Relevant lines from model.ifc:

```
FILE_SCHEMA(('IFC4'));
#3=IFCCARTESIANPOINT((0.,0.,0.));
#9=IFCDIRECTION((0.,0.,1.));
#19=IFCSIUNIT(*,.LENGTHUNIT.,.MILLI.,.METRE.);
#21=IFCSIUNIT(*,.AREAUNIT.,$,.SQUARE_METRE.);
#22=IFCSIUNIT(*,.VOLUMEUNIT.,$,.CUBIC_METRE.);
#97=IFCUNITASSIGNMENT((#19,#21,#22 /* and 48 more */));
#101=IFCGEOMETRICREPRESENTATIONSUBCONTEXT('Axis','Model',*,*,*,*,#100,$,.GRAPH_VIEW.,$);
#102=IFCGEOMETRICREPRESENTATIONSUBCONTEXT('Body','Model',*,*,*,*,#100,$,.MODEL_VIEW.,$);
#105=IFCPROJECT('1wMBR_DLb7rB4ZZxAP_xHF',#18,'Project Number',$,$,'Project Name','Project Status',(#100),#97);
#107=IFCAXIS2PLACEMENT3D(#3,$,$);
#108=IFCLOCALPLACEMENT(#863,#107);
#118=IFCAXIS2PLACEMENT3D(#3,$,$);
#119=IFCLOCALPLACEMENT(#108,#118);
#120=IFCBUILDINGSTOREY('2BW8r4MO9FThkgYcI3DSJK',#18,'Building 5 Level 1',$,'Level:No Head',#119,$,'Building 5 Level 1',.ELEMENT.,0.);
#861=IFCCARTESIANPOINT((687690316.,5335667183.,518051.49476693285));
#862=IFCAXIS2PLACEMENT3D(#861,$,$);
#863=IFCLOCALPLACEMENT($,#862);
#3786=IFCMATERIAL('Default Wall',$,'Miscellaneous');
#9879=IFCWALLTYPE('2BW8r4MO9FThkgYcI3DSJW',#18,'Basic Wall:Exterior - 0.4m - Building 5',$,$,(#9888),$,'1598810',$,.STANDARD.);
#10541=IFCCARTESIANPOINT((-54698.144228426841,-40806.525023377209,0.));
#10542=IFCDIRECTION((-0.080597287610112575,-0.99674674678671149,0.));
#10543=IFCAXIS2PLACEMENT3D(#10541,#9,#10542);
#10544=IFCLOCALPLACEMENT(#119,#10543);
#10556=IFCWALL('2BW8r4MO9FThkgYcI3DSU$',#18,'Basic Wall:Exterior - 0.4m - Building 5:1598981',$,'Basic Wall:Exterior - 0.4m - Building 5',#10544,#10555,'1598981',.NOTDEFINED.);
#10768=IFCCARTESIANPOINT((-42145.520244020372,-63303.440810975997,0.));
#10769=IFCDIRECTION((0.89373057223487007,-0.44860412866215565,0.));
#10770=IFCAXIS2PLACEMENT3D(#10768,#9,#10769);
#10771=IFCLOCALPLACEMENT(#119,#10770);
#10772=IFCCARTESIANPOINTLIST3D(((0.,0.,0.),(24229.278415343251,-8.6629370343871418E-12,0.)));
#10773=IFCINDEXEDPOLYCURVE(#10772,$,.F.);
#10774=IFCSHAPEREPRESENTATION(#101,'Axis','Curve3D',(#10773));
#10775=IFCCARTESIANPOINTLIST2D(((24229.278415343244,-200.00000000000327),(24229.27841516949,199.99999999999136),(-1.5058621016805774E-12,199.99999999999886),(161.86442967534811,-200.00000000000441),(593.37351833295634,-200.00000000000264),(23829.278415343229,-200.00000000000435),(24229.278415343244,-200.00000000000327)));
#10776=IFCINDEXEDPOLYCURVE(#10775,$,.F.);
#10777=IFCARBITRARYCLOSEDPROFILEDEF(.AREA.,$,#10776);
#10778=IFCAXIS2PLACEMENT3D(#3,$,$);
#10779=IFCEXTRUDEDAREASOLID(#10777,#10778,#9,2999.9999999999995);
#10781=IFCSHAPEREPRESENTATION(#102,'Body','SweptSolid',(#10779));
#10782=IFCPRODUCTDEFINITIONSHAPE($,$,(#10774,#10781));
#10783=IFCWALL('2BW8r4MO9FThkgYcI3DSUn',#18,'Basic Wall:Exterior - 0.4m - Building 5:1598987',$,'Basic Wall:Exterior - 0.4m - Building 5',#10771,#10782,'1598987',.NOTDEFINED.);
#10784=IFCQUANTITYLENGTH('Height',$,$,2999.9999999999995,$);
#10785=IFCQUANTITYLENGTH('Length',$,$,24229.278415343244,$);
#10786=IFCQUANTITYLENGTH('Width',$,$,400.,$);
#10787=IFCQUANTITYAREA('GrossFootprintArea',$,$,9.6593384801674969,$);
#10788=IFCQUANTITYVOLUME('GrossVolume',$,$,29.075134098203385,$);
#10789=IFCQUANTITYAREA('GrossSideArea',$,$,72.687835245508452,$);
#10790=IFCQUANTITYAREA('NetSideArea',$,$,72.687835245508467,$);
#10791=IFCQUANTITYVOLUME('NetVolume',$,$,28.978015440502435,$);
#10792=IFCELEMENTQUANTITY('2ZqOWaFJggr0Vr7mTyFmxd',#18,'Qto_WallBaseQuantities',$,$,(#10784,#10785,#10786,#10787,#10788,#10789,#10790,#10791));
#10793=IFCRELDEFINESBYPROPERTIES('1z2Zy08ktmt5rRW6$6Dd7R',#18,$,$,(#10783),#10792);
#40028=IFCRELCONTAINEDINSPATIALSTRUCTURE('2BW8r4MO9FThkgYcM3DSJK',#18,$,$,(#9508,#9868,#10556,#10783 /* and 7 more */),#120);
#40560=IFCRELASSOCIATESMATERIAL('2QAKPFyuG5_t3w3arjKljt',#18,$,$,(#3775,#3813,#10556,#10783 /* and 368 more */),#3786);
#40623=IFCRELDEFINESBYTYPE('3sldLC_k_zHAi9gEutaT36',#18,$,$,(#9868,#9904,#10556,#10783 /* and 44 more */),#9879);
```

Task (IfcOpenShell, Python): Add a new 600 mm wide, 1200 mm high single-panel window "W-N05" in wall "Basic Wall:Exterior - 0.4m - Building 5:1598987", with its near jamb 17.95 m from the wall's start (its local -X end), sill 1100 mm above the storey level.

```python
import numpy as np
import ifcopenshell
import ifcopenshell.api.feature
import ifcopenshell.api.geometry
import ifcopenshell.api.pset
import ifcopenshell.api.root
import ifcopenshell.api.spatial
import ifcopenshell.geom
import ifcopenshell.util.element
import ifcopenshell.util.placement
import ifcopenshell.util.representation
import ifcopenshell.util.shape
import ifcopenshell.util.unit

model = ifcopenshell.open("model.ifc")
unit_scale = ifcopenshell.util.unit.calculate_unit_scale(model)
area_scale = ifcopenshell.util.unit.calculate_unit_scale(model, "AREAUNIT")
volume_scale = ifcopenshell.util.unit.calculate_unit_scale(model, "VOLUMEUNIT")
settings = ifcopenshell.geom.settings()


def volume(element):
    """Net volume in cubic metres, openings subtracted."""
    shape = ifcopenshell.geom.create_shape(settings, element)
    return ifcopenshell.util.shape.get_volume(shape.geometry)


wall = model.by_guid("2BW8r4MO9FThkgYcI3DSUn")
storey = ifcopenshell.util.element.get_container(wall, ifc_class="IfcBuildingStorey")
context = ifcopenshell.util.representation.get_context(model, "Model", "Body", "MODEL_VIEW")
before = volume(wall)

width, height, from_end, sill = 0.6, 1.2, 17.95, 1.1  # metres

# The wall runs along its own X axis, and the end named is its -X end.
wall_shape = ifcopenshell.geom.create_shape(settings, wall)
x, y, z = ifcopenshell.util.shape.get_vertices(wall_shape.geometry).T
start = x.min() + from_end
face, thickness = float(y.min()), float(y.max() - y.min())
wall_matrix = ifcopenshell.util.placement.get_local_placement(wall.ObjectPlacement)
level = ifcopenshell.util.placement.get_local_placement(storey.ObjectPlacement)[2, 3]


def in_wall(x, y):
    """Placement at x, y metres in the wall's axes, at sill height."""
    matrix = wall_matrix.copy()
    matrix[:, 3] = wall_matrix @ np.array([x / unit_scale, y / unit_scale, 0.0, 1.0])
    matrix[2, 3] = level + sill / unit_scale
    return matrix


# Opening: a box that overshoots both wall faces by 50 mm.
opening = ifcopenshell.api.root.create_entity(model, ifc_class="IfcOpeningElement", predefined_type="OPENING")
box = ifcopenshell.api.geometry.add_wall_representation(
    model, context=context, length=width, height=height, thickness=thickness + 0.1
)
ifcopenshell.api.geometry.assign_representation(model, product=opening, representation=box)
ifcopenshell.api.geometry.edit_object_placement(model, product=opening, matrix=in_wall(start, face - 0.05), is_si=False)
ifcopenshell.api.feature.add_feature(model, feature=opening, element=wall)

window = ifcopenshell.api.root.create_entity(model, ifc_class="IfcWindow", name="W-N05", predefined_type="WINDOW")
window.OverallWidth, window.OverallHeight = width / unit_scale, height / unit_scale
window.PartitioningType = "SINGLE_PANEL"
body = ifcopenshell.api.geometry.add_window_representation(
    model,
    context=context,
    overall_width=window.OverallWidth,
    overall_height=window.OverallHeight,
    partition_type="SINGLE_PANEL",
)
ifcopenshell.api.geometry.assign_representation(model, product=window, representation=body)
ifcopenshell.api.spatial.assign_container(model, products=[window], relating_structure=storey)
ifcopenshell.api.feature.add_filling(model, opening=opening, element=window)

# Centre the window in the wall's thickness.
ifcopenshell.api.geometry.edit_object_placement(model, product=window, matrix=in_wall(start, face), is_si=False)
window_shape = ifcopenshell.geom.create_shape(settings, window)
depth = ifcopenshell.util.shape.get_vertices(window_shape.geometry)[:, 1]
offset = face + thickness / 2 - (depth.min() + depth.max()) / 2
ifcopenshell.api.geometry.edit_object_placement(model, product=window, matrix=in_wall(start, offset), is_si=False)

after = volume(wall)

# Update the wall's stored quantities.
qto = model.by_id(ifcopenshell.util.element.get_pset(wall, "Qto_WallBaseQuantities", should_inherit=False)["id"])
ifcopenshell.api.pset.edit_qto(model, qto=qto, properties={
    "NetSideArea": after / thickness / area_scale,
    "NetVolume": after / volume_scale,
})

print(f"wall volume {before:.3f} -> {after:.3f} m3")

model.write("model_v2.ifc")
```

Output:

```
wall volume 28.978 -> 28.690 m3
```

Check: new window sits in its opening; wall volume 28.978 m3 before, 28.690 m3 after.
